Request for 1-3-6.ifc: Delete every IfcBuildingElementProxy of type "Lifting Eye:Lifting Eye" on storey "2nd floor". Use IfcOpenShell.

First a look at what the model holds.

```python
import ifcopenshell
import ifcopenshell.util.element

model = ifcopenshell.open("1-3-6.ifc")
print(model.schema)
storey = next(s for s in model.by_type("IfcBuildingStorey") if s.Name == "2nd floor")
proxies = [e for e in ifcopenshell.util.element.get_decomposition(storey) if e.is_a("IfcBuildingElementProxy")]
seen = {}
for e in proxies:
    element_type = ifcopenshell.util.element.get_type(e)
    name = element_type.Name if element_type not in (None, e) else None
    seen[name] = seen.get(name, 0) + 1
for name, count in sorted(seen.items(), key=str):
    print(count, "x", name)
```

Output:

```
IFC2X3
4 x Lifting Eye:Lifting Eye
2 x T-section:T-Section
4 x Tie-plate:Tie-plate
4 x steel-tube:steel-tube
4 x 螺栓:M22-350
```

```python
import ifcopenshell
import ifcopenshell.api.root
import ifcopenshell.util.element

model = ifcopenshell.open("1-3-6.ifc")

storey = next(s for s in model.by_type("IfcBuildingStorey") if s.Name == "2nd floor")
proxies = [e for e in ifcopenshell.util.element.get_decomposition(storey) if e.is_a("IfcBuildingElementProxy")]
targets = [e for e in proxies if (t := ifcopenshell.util.element.get_type(e)) not in (None, e) and t.Name == "Lifting Eye:Lifting Eye"]

for e in targets:
    ifcopenshell.api.root.remove_product(model, product=e)
print(len(targets), "removed")

model.write("1-3-6_edited.ifc")
```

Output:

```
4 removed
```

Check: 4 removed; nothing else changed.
